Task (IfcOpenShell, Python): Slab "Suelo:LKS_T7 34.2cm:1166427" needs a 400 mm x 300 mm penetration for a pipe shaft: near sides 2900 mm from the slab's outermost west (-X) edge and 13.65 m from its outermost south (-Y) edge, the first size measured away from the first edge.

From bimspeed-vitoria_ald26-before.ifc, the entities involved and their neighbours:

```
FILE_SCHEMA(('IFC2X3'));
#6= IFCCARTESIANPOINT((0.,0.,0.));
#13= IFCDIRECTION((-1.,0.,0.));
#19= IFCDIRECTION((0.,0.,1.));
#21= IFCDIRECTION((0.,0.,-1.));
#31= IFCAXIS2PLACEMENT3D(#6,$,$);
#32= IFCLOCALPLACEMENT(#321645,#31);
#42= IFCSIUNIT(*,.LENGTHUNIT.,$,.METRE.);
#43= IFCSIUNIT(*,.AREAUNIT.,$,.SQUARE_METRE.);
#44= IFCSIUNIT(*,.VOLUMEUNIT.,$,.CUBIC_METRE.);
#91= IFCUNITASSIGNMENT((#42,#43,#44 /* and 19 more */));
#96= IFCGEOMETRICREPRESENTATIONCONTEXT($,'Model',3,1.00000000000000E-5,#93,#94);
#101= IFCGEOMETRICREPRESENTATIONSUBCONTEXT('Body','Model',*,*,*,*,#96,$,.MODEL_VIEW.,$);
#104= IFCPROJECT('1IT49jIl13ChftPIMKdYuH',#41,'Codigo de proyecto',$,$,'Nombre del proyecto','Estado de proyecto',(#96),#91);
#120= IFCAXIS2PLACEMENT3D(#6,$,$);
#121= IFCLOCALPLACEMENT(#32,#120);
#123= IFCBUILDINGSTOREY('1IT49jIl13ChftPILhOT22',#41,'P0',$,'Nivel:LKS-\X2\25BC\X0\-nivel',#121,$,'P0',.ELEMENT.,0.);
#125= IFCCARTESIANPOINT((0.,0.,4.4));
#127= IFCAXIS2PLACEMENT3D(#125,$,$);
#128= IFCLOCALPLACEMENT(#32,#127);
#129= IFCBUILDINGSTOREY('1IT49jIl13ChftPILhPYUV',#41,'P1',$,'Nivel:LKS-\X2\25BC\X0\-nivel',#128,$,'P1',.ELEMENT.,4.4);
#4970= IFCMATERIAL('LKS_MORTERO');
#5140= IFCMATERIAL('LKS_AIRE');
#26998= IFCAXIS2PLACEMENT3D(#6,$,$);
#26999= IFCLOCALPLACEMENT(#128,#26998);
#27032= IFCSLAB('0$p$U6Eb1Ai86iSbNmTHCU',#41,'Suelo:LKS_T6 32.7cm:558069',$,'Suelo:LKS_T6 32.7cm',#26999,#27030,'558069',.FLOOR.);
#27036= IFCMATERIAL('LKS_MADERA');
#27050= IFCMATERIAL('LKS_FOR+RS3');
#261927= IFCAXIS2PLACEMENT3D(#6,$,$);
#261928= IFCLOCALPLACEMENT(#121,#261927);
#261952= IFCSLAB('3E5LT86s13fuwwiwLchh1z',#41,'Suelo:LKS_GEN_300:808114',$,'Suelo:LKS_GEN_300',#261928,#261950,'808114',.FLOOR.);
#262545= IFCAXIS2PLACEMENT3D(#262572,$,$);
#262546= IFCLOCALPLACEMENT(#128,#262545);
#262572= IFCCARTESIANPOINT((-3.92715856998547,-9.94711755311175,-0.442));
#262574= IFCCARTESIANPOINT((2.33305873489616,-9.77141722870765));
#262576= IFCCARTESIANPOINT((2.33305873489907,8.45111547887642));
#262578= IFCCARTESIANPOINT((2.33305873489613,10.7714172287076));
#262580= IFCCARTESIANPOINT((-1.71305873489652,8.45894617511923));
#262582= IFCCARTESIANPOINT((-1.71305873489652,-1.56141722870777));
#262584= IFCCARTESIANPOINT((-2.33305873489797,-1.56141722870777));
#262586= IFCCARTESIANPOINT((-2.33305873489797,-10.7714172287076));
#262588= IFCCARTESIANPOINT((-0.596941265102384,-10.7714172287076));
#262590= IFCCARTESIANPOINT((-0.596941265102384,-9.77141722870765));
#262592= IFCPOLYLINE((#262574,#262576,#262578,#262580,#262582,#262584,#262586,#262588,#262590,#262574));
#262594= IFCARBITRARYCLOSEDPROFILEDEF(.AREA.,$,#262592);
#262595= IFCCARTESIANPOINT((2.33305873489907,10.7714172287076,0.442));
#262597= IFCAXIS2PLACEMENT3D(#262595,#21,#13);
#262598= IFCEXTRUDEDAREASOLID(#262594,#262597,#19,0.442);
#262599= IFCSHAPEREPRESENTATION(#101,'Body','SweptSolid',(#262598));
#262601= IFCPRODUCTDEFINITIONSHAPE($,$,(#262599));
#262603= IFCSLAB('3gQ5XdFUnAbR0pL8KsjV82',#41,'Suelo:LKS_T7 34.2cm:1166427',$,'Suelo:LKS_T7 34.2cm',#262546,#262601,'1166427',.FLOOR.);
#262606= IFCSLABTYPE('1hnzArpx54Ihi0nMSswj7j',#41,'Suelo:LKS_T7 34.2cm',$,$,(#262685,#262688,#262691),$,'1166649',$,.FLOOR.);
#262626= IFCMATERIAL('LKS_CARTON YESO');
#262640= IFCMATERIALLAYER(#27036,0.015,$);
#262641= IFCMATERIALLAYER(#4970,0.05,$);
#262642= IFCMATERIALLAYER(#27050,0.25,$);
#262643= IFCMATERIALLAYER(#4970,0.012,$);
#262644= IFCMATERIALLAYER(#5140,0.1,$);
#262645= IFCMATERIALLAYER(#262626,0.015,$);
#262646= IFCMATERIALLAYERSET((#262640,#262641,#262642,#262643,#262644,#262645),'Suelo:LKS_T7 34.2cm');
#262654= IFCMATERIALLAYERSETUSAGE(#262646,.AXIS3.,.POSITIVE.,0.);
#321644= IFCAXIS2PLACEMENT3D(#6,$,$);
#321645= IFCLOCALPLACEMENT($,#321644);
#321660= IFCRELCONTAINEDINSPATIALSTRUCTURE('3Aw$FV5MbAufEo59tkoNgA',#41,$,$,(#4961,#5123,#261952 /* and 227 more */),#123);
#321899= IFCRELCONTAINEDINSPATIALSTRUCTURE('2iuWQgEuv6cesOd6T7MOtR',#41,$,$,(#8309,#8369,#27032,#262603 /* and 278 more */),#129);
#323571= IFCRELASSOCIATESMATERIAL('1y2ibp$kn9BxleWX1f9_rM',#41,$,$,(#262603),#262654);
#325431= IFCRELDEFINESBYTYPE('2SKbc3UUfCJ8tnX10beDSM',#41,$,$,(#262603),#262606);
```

```python
import numpy as np
import ifcopenshell
import ifcopenshell.api.feature
import ifcopenshell.api.geometry
import ifcopenshell.api.root
import ifcopenshell.geom
import ifcopenshell.util.placement
import ifcopenshell.util.representation
import ifcopenshell.util.shape
import ifcopenshell.util.unit

model = ifcopenshell.open("bimspeed-vitoria_ald26-before.ifc")
unit_scale = ifcopenshell.util.unit.calculate_unit_scale(model)
settings = ifcopenshell.geom.settings()


def volume(element):
    """Net volume in cubic metres, openings subtracted."""
    shape = ifcopenshell.geom.create_shape(settings, element)
    return ifcopenshell.util.shape.get_volume(shape.geometry)


slab = model.by_guid("3gQ5XdFUnAbR0pL8KsjV82")
before = volume(slab)

# Extent in the slab's own axes, in metres. The edges named are its -X and -Y sides.
slab_shape = ifcopenshell.geom.create_shape(settings, slab)
vertices = ifcopenshell.util.shape.get_vertices(slab_shape.geometry)
x_min, y_min, bottom = vertices.min(axis=0)
top = vertices[:, 2].max()

opening = ifcopenshell.api.root.create_entity(model, ifc_class="IfcOpeningElement", name="Pipe shaft opening")
context = ifcopenshell.util.representation.get_context(model, "Model", "Body", "MODEL_VIEW")
width, depth = 0.4, 0.3
outline = [(0.0, 0.0), (width, 0.0), (width, depth), (0.0, depth), (0.0, 0.0)]
# Overshoot both faces by 50 mm so the cut is clean.
shape = ifcopenshell.api.geometry.add_slab_representation(
    model, context=context, depth=top - bottom + 0.1, polyline=outline
)
ifcopenshell.api.geometry.assign_representation(model, product=opening, representation=shape)

matrix = ifcopenshell.util.placement.get_local_placement(slab.ObjectPlacement)
matrix[:, 3] = matrix @ np.append(np.array([x_min + 2.9, y_min + 13.65, bottom - 0.05]) / unit_scale, 1.0)
ifcopenshell.api.geometry.edit_object_placement(model, product=opening, matrix=matrix, is_si=False)
ifcopenshell.api.feature.add_feature(model, feature=opening, element=slab)

after = volume(slab)

print(f"slab volume {before:.3f} -> {after:.3f} m3")

model.write("bimspeed-vitoria_ald26-before-out.ifc")
```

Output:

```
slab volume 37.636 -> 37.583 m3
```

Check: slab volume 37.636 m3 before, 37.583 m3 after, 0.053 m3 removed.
